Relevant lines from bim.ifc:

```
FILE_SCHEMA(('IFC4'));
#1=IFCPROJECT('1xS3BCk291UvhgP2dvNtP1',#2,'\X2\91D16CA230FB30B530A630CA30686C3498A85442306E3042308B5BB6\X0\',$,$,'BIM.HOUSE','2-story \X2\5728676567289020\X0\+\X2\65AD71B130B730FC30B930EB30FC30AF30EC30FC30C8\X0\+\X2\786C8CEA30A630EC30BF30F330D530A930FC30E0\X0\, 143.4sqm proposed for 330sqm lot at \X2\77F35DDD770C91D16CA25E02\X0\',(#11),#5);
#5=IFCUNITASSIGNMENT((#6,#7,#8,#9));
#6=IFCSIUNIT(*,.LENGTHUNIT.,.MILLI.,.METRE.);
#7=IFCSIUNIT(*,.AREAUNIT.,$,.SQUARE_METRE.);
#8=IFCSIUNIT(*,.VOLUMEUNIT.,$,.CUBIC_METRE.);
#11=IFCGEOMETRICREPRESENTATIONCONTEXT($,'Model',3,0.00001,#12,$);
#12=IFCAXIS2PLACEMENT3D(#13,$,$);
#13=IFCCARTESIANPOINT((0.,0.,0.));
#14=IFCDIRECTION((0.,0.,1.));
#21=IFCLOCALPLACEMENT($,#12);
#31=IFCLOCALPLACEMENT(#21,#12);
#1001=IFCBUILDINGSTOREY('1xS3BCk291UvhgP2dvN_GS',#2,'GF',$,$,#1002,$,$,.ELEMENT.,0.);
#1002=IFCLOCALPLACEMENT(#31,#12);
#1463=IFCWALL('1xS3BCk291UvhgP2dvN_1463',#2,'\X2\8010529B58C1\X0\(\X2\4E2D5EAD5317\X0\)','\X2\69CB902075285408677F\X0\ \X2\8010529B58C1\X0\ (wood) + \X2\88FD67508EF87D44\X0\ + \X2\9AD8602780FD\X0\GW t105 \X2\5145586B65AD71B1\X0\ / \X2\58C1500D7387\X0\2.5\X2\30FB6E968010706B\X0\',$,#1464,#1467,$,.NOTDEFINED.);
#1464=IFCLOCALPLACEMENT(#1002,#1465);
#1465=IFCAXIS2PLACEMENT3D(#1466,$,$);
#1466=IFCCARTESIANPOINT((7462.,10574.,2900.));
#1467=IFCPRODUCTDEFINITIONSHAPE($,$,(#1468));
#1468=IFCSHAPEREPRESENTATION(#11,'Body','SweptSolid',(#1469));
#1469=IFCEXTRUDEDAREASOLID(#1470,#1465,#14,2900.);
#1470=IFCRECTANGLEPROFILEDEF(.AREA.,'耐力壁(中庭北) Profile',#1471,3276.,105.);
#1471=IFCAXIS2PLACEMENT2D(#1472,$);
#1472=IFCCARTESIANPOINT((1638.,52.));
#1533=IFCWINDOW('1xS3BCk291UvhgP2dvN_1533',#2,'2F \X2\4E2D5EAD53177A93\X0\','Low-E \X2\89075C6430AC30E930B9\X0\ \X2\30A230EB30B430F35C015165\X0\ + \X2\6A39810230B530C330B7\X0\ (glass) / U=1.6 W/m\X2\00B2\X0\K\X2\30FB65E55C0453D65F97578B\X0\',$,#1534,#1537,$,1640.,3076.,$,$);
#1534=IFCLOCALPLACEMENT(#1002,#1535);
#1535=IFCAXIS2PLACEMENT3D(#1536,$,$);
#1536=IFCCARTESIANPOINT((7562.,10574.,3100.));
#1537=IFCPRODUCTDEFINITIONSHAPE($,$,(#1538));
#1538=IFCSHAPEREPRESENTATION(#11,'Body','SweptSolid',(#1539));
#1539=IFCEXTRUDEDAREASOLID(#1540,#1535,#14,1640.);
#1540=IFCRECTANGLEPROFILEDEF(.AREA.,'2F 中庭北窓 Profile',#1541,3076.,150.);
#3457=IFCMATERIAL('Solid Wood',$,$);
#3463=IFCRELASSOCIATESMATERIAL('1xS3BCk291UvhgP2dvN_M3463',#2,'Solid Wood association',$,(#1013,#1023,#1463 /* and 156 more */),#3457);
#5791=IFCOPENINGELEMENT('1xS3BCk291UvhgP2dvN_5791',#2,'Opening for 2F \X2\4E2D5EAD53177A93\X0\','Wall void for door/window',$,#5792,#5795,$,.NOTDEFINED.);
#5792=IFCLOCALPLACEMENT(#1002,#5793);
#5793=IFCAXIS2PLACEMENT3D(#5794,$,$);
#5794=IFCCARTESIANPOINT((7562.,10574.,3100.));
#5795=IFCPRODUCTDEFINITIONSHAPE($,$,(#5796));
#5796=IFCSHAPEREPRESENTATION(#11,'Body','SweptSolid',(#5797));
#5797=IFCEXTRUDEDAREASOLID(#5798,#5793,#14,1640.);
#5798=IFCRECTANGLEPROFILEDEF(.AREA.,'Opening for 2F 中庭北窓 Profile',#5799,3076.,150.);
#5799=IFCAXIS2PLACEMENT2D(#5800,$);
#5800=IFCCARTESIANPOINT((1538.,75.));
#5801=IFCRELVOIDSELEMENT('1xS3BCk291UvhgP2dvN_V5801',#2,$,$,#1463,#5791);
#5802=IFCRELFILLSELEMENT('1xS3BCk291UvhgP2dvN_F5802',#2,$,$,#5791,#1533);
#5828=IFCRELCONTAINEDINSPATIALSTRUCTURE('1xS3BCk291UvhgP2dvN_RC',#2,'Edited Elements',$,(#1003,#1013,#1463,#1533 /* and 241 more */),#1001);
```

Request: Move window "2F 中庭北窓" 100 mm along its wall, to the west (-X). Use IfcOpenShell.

```python
import ifcopenshell
import ifcopenshell.api.geometry
import ifcopenshell.util.placement
import ifcopenshell.util.unit

model = ifcopenshell.open("bim.ifc")
unit_scale = ifcopenshell.util.unit.calculate_unit_scale(model)

window = model.by_guid("1xS3BCk291UvhgP2dvN_1533")
opening = window.FillsVoids[0].RelatingOpeningElement
wall = opening.VoidsElements[0].RelatingBuildingElement

wall_matrix = ifcopenshell.util.placement.get_local_placement(wall.ObjectPlacement)
shift = wall_matrix[:3, 0] * -0.1 / unit_scale
before = ifcopenshell.util.placement.get_local_placement(window.ObjectPlacement)[:3, 3].copy()

# The window is not placed relative to its opening, so move both.
for product in (opening, window):
    matrix = ifcopenshell.util.placement.get_local_placement(product.ObjectPlacement)
    matrix[:3, 3] += shift
    ifcopenshell.api.geometry.edit_object_placement(model, product=product, matrix=matrix, is_si=False)

after = ifcopenshell.util.placement.get_local_placement(window.ObjectPlacement)[:3, 3]
print("window moved by", (after - before).round(3) + 0.0)

model.write("bim_v2.ifc")
```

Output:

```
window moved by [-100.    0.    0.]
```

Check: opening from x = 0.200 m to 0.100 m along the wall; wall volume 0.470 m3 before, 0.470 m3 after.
